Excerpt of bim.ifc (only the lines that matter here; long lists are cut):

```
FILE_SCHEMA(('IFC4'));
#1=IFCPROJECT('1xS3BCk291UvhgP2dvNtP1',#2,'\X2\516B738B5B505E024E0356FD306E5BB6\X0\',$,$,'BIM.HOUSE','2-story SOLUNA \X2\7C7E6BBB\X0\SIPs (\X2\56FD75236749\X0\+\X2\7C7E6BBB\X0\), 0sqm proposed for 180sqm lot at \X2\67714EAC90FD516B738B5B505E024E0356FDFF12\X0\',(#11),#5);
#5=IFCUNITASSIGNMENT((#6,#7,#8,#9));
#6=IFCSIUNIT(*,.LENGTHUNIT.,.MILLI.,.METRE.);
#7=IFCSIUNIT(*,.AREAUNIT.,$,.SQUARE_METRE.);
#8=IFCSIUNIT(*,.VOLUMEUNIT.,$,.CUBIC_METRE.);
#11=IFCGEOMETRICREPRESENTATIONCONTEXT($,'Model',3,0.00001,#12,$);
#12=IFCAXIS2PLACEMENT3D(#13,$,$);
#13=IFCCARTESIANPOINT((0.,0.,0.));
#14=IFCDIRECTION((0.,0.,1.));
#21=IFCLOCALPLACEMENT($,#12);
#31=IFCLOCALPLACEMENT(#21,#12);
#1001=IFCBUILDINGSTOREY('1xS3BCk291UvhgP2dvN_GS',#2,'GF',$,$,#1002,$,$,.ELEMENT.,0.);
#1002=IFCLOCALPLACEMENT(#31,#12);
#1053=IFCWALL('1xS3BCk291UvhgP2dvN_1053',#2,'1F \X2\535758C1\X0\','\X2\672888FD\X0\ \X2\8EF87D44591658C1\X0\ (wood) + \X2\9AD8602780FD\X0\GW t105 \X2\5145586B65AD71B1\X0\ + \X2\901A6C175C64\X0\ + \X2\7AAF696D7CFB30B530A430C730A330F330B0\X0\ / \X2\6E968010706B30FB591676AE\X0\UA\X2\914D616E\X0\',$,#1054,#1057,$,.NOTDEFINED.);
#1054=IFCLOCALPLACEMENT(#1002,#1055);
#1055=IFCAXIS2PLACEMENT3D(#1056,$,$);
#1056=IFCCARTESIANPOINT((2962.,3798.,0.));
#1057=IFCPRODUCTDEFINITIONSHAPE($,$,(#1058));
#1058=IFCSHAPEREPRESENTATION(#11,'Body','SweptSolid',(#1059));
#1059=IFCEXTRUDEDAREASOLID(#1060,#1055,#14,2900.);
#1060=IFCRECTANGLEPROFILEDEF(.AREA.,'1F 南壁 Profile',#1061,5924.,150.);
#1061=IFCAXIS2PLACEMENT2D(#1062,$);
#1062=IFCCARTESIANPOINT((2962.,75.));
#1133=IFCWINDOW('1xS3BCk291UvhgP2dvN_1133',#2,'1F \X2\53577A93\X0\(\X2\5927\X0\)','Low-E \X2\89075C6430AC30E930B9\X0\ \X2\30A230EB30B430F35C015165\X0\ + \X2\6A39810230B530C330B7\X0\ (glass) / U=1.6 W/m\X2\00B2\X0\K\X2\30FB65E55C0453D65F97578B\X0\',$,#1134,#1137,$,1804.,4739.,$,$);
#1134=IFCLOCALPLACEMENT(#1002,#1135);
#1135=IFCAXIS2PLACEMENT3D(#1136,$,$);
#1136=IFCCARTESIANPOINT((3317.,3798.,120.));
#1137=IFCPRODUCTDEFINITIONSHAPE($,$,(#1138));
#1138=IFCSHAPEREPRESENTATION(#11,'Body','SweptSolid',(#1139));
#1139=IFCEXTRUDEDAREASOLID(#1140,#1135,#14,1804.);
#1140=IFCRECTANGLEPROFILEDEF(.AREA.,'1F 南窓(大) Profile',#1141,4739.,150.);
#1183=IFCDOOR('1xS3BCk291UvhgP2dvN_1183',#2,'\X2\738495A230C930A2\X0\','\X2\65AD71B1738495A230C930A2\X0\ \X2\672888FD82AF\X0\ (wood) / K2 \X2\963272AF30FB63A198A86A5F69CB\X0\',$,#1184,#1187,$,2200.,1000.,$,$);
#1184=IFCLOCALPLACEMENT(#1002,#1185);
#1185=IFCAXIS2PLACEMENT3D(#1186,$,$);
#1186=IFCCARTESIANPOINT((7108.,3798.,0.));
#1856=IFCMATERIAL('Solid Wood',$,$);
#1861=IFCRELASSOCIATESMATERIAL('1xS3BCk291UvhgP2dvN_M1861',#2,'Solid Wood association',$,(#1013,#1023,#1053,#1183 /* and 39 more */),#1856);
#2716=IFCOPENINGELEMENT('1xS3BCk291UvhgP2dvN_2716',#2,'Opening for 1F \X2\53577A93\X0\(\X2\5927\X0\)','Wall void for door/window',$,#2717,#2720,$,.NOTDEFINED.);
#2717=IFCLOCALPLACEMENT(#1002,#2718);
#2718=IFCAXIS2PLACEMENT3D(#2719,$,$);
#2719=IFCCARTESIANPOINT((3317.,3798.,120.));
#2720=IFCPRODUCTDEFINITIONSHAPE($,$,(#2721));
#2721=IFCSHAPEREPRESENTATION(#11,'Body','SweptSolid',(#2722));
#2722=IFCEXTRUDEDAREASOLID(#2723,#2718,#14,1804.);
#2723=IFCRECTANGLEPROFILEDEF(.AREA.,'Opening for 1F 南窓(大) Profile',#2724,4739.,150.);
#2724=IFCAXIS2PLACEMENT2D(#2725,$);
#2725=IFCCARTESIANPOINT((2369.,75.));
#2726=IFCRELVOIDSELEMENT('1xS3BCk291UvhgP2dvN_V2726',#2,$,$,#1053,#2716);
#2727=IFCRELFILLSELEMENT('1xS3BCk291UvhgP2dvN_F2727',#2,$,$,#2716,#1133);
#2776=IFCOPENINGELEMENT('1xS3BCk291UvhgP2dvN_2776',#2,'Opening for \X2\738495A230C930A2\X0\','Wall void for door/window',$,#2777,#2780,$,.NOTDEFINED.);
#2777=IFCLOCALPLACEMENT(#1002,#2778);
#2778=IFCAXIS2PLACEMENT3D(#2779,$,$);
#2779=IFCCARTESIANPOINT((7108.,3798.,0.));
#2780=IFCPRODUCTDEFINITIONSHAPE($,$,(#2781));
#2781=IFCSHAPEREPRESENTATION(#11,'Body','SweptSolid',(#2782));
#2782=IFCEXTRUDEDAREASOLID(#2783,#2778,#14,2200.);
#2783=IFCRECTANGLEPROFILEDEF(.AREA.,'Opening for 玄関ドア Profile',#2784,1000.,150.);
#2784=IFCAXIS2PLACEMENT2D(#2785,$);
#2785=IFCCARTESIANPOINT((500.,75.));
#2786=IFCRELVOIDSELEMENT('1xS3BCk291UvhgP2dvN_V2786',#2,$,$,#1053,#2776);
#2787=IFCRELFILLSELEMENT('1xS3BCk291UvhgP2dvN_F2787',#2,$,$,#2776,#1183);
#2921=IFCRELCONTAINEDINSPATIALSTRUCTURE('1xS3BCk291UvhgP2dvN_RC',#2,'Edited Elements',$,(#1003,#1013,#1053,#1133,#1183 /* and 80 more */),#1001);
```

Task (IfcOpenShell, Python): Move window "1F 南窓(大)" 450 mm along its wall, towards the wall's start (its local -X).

```python
import ifcopenshell
import ifcopenshell.api.geometry
import ifcopenshell.util.placement
import ifcopenshell.util.unit

model = ifcopenshell.open("bim.ifc")
unit_scale = ifcopenshell.util.unit.calculate_unit_scale(model)

window = model.by_id(1133)
opening = window.FillsVoids[0].RelatingOpeningElement
wall = opening.VoidsElements[0].RelatingBuildingElement

wall_matrix = ifcopenshell.util.placement.get_local_placement(wall.ObjectPlacement)
shift = wall_matrix[:3, 0] * -0.45 / unit_scale
before = ifcopenshell.util.placement.get_local_placement(window.ObjectPlacement)[:3, 3].copy()

# The window is not placed relative to its opening, so move both.
for product in (opening, window):
    matrix = ifcopenshell.util.placement.get_local_placement(product.ObjectPlacement)
    matrix[:3, 3] += shift
    ifcopenshell.api.geometry.edit_object_placement(model, product=product, matrix=matrix, is_si=False)

after = ifcopenshell.util.placement.get_local_placement(window.ObjectPlacement)[:3, 3]
print("window moved by", (after - before).round(3) + 0.0)

model.write("bim_updated.ifc")
```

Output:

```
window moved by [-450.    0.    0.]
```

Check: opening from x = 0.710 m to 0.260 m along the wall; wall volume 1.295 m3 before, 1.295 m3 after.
